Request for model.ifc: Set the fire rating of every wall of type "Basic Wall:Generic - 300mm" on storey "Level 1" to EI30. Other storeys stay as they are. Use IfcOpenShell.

First a look at what the model holds.

```python
import ifcopenshell
import ifcopenshell.util.element

model = ifcopenshell.open("model.ifc")
print(model.schema)
storey = next(s for s in model.by_type("IfcBuildingStorey") if s.Name == "Level 1")
walls = [e for e in ifcopenshell.util.element.get_decomposition(storey) if e.is_a("IfcWall")]
seen = {}
for e in walls:
    element_type = ifcopenshell.util.element.get_type(e)
    key = (element_type.Name if element_type != e and element_type else None, ifcopenshell.util.element.get_pset(e, "Pset_WallCommon", "FireRating"))
    seen[key] = seen.get(key, 0) + 1
for (name, value), count in sorted(seen.items(), key=str):
    print(count, "x", name, "|", value)
```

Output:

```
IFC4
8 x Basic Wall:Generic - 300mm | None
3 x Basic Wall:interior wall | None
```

```python
import ifcopenshell
import ifcopenshell.api.pset
import ifcopenshell.util.element

model = ifcopenshell.open("model.ifc")

storey = next(s for s in model.by_type("IfcBuildingStorey") if s.Name == "Level 1")
walls = [e for e in ifcopenshell.util.element.get_decomposition(storey) if e.is_a("IfcWall")]

count = 0
for e in walls:
    element_type = ifcopenshell.util.element.get_type(e)
    if element_type in (None, e) or element_type.Name != "Basic Wall:Generic - 300mm":
        continue
    # add_pset returns the element's existing set when there is one.
    pset = ifcopenshell.api.pset.add_pset(model, product=e, name="Pset_WallCommon")
    ifcopenshell.api.pset.edit_pset(model, pset=pset, properties={"FireRating": "EI30"})
    count += 1

print(count, "walls updated")

model.write("model_v2.ifc")
```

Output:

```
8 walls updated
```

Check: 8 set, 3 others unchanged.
